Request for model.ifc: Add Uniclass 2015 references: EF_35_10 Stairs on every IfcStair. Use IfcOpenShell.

First a look at what the model holds.

```python
import ifcopenshell

model = ifcopenshell.open("model.ifc")
print(model.schema)
print("classifications:", [c.Name for c in model.by_type("IfcClassification")])
for ifc_class in ("IfcDoor", "IfcRoof", "IfcStair", "IfcWall", "IfcWindow"):
    print(ifc_class, len(model.by_type(ifc_class)))
```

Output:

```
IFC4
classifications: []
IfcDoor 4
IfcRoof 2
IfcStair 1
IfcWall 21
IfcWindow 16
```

```python
import ifcopenshell
import ifcopenshell.api.classification

model = ifcopenshell.open("model.ifc")

system = ifcopenshell.api.classification.add_classification(model, classification="Uniclass 2015")

codes = {
    "IfcStair": ("EF_35_10", "Stairs"),
}
for ifc_class, (code, name) in codes.items():
    products = model.by_type(ifc_class)
    ifcopenshell.api.classification.add_reference(
        model, products=products, classification=system, identification=code, name=name
    )
    print(code, len(products))

model.write("model-out.ifc")
```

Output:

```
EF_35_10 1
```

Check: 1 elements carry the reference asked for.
